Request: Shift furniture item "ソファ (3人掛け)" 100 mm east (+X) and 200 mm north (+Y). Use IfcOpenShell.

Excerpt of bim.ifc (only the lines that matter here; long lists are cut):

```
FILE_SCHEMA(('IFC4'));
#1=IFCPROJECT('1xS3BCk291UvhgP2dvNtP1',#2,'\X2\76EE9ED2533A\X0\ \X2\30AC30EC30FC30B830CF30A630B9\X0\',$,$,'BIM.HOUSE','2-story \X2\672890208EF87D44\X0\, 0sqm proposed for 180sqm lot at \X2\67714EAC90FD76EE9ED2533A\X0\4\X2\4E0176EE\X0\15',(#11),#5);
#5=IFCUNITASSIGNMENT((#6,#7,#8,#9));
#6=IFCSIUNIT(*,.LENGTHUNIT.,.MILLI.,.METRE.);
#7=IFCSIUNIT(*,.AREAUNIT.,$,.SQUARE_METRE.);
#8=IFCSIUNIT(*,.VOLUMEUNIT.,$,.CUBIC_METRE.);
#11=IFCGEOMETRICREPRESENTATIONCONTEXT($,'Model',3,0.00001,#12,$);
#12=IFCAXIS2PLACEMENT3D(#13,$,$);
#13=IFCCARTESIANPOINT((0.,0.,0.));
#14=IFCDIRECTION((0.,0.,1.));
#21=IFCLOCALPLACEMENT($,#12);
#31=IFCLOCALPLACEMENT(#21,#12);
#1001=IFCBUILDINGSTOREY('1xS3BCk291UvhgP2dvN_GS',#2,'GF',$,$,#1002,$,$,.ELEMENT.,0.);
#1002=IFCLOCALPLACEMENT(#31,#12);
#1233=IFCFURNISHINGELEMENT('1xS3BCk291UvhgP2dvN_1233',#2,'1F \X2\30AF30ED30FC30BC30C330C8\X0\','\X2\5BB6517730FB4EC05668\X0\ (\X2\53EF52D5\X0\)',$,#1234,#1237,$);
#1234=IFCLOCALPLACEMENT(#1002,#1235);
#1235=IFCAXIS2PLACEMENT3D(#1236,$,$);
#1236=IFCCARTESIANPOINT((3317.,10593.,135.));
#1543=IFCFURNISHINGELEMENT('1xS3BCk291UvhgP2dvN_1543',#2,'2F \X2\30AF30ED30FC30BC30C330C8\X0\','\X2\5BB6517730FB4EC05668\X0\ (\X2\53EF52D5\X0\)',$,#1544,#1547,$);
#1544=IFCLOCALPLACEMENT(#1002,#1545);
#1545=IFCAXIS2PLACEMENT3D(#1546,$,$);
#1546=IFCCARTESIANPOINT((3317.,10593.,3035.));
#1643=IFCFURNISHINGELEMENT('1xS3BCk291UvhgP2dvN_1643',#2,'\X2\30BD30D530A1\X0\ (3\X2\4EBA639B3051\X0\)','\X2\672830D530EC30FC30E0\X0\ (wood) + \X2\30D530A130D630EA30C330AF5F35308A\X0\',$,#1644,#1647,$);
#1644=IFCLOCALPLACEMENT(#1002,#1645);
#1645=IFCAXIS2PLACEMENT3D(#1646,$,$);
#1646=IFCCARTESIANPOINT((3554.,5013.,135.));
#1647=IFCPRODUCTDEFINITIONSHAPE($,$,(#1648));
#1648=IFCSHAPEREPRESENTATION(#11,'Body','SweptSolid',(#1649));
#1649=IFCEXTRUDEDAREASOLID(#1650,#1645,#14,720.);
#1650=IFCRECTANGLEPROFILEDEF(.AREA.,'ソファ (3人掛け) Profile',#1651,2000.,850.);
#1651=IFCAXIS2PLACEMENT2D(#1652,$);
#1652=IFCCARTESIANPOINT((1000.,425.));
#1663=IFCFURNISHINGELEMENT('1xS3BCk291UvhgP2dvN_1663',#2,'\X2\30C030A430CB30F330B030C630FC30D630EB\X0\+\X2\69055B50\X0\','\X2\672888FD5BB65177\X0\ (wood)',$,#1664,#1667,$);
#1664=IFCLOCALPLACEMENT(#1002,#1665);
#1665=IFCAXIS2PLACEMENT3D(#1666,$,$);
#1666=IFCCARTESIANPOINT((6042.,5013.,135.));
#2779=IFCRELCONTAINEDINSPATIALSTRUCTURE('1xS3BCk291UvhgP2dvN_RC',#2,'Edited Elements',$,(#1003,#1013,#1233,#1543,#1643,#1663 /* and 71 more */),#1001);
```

```python
import ifcopenshell
import ifcopenshell.api.geometry
import ifcopenshell.util.placement

model = ifcopenshell.open("bim.ifc")

item = model.by_guid("1xS3BCk291UvhgP2dvN_1643")
matrix = ifcopenshell.util.placement.get_local_placement(item.ObjectPlacement)
matrix[0, 3] += 100.0
matrix[1, 3] += 200.0
ifcopenshell.api.geometry.edit_object_placement(model, product=item, matrix=matrix, is_si=False)

print(ifcopenshell.util.placement.get_local_placement(item.ObjectPlacement).round(3) + 0.0)

model.write("bim_rev.ifc")
```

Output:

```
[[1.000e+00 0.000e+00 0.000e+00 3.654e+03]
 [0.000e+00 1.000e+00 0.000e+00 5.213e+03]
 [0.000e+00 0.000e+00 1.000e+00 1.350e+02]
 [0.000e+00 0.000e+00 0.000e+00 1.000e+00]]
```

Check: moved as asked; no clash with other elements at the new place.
